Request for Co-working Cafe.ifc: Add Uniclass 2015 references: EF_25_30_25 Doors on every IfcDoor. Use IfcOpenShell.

First a look at what the model holds.

```python
import ifcopenshell

model = ifcopenshell.open("Co-working Cafe.ifc")
print(model.schema)
print("classifications:", [c.Name for c in model.by_type("IfcClassification")])
for ifc_class in ("IfcDoor", "IfcRoof", "IfcStair", "IfcWall", "IfcWindow"):
    print(ifc_class, len(model.by_type(ifc_class)))
```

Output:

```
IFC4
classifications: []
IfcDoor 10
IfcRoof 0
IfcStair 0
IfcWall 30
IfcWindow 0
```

```python
import ifcopenshell
import ifcopenshell.api.classification

model = ifcopenshell.open("Co-working Cafe.ifc")

system = ifcopenshell.api.classification.add_classification(model, classification="Uniclass 2015")

codes = {
    "IfcDoor": ("EF_25_30_25", "Doors"),
}
for ifc_class, (code, name) in codes.items():
    products = model.by_type(ifc_class)
    ifcopenshell.api.classification.add_reference(
        model, products=products, classification=system, identification=code, name=name
    )
    print(code, len(products))

model.write("Co-working Cafe_edited.ifc")
```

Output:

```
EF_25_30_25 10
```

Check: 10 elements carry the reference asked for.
